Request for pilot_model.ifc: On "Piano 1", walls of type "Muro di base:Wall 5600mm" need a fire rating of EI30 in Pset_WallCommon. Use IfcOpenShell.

First a look at what the model holds.

```python
import ifcopenshell
import ifcopenshell.util.element

model = ifcopenshell.open("pilot_model.ifc")
print(model.schema)
storey = next(s for s in model.by_type("IfcBuildingStorey") if s.Name == "Piano 1")
walls = [e for e in ifcopenshell.util.element.get_decomposition(storey) if e.is_a("IfcWall")]
seen = {}
for e in walls:
    element_type = ifcopenshell.util.element.get_type(e)
    key = (element_type.Name if element_type != e and element_type else None, ifcopenshell.util.element.get_pset(e, "Pset_WallCommon", "FireRating"))
    seen[key] = seen.get(key, 0) + 1
for (name, value), count in sorted(seen.items(), key=str):
    print(count, "x", name, "|", value)
```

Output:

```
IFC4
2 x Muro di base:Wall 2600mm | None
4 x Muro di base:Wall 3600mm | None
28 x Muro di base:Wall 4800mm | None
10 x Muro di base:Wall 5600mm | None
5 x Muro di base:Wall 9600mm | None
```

```python
import ifcopenshell
import ifcopenshell.api.pset
import ifcopenshell.util.element

model = ifcopenshell.open("pilot_model.ifc")

storey = next(s for s in model.by_type("IfcBuildingStorey") if s.Name == "Piano 1")
walls = [e for e in ifcopenshell.util.element.get_decomposition(storey) if e.is_a("IfcWall")]

count = 0
for e in walls:
    element_type = ifcopenshell.util.element.get_type(e)
    if element_type in (None, e) or element_type.Name != "Muro di base:Wall 5600mm":
        continue
    # add_pset returns the element's existing set when there is one.
    pset = ifcopenshell.api.pset.add_pset(model, product=e, name="Pset_WallCommon")
    ifcopenshell.api.pset.edit_pset(model, pset=pset, properties={"FireRating": "EI30"})
    count += 1

print(count, "walls updated")

model.write("pilot_model-out.ifc")
```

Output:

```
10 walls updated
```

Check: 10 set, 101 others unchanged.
